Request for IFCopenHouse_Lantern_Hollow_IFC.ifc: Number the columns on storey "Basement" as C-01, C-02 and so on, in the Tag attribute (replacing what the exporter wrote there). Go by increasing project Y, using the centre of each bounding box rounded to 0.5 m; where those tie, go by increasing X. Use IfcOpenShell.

First a look at what the model holds.

```python
import ifcopenshell
import ifcopenshell.util.element
import ifcopenshell.util.placement

model = ifcopenshell.open("IFCopenHouse_Lantern_Hollow_IFC.ifc")
print(model.schema)
storey = next(s for s in model.by_type("IfcBuildingStorey") if s.Name == "Basement")
columns = [e for e in ifcopenshell.util.element.get_decomposition(storey) if e.is_a("IfcColumn")]
for e in sorted(columns, key=lambda e: e.id()):
    origin = ifcopenshell.util.placement.get_local_placement(e.ObjectPlacement)[:3, 3]
    print(e.id(), e.Tag, e.Name, origin.round(2) + 0.0, sep=" | ")
```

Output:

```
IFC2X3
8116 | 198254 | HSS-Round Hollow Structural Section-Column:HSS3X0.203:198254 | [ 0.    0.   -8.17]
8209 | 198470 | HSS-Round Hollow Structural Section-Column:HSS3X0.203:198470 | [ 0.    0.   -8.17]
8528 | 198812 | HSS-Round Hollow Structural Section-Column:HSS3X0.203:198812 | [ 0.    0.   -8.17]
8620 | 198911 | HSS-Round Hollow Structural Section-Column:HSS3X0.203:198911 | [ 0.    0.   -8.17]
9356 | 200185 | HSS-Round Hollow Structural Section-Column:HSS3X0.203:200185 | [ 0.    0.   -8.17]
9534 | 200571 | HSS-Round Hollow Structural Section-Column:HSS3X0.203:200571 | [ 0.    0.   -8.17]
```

```python
import ifcopenshell
import ifcopenshell.geom
import ifcopenshell.util.element
import ifcopenshell.util.shape

model = ifcopenshell.open("IFCopenHouse_Lantern_Hollow_IFC.ifc")
settings = ifcopenshell.geom.settings()
settings.set("use-world-coords", True)


def centre(element):
    shape = ifcopenshell.geom.create_shape(settings, element)
    return ifcopenshell.util.shape.get_bbox_centroid(shape.geometry)


storey = next(s for s in model.by_type("IfcBuildingStorey") if s.Name == "Basement")
columns = [e for e in ifcopenshell.util.element.get_decomposition(storey) if e.is_a("IfcColumn")]

# Insertion points can sit at a corner or the storey origin, so sort by the geometry (in metres).
centres = {e: centre(e) for e in columns}
columns.sort(key=lambda e: (round(centres[e][1] / 0.5), centres[e][0]))

for i, e in enumerate(columns, start=1):
    number = f"C-{i:02d}"
    e.Tag = number
    print(e.id(), number)

model.write("IFCopenHouse_Lantern_Hollow_IFC_v2.ifc")
```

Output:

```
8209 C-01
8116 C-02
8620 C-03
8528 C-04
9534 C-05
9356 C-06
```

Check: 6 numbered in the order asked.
